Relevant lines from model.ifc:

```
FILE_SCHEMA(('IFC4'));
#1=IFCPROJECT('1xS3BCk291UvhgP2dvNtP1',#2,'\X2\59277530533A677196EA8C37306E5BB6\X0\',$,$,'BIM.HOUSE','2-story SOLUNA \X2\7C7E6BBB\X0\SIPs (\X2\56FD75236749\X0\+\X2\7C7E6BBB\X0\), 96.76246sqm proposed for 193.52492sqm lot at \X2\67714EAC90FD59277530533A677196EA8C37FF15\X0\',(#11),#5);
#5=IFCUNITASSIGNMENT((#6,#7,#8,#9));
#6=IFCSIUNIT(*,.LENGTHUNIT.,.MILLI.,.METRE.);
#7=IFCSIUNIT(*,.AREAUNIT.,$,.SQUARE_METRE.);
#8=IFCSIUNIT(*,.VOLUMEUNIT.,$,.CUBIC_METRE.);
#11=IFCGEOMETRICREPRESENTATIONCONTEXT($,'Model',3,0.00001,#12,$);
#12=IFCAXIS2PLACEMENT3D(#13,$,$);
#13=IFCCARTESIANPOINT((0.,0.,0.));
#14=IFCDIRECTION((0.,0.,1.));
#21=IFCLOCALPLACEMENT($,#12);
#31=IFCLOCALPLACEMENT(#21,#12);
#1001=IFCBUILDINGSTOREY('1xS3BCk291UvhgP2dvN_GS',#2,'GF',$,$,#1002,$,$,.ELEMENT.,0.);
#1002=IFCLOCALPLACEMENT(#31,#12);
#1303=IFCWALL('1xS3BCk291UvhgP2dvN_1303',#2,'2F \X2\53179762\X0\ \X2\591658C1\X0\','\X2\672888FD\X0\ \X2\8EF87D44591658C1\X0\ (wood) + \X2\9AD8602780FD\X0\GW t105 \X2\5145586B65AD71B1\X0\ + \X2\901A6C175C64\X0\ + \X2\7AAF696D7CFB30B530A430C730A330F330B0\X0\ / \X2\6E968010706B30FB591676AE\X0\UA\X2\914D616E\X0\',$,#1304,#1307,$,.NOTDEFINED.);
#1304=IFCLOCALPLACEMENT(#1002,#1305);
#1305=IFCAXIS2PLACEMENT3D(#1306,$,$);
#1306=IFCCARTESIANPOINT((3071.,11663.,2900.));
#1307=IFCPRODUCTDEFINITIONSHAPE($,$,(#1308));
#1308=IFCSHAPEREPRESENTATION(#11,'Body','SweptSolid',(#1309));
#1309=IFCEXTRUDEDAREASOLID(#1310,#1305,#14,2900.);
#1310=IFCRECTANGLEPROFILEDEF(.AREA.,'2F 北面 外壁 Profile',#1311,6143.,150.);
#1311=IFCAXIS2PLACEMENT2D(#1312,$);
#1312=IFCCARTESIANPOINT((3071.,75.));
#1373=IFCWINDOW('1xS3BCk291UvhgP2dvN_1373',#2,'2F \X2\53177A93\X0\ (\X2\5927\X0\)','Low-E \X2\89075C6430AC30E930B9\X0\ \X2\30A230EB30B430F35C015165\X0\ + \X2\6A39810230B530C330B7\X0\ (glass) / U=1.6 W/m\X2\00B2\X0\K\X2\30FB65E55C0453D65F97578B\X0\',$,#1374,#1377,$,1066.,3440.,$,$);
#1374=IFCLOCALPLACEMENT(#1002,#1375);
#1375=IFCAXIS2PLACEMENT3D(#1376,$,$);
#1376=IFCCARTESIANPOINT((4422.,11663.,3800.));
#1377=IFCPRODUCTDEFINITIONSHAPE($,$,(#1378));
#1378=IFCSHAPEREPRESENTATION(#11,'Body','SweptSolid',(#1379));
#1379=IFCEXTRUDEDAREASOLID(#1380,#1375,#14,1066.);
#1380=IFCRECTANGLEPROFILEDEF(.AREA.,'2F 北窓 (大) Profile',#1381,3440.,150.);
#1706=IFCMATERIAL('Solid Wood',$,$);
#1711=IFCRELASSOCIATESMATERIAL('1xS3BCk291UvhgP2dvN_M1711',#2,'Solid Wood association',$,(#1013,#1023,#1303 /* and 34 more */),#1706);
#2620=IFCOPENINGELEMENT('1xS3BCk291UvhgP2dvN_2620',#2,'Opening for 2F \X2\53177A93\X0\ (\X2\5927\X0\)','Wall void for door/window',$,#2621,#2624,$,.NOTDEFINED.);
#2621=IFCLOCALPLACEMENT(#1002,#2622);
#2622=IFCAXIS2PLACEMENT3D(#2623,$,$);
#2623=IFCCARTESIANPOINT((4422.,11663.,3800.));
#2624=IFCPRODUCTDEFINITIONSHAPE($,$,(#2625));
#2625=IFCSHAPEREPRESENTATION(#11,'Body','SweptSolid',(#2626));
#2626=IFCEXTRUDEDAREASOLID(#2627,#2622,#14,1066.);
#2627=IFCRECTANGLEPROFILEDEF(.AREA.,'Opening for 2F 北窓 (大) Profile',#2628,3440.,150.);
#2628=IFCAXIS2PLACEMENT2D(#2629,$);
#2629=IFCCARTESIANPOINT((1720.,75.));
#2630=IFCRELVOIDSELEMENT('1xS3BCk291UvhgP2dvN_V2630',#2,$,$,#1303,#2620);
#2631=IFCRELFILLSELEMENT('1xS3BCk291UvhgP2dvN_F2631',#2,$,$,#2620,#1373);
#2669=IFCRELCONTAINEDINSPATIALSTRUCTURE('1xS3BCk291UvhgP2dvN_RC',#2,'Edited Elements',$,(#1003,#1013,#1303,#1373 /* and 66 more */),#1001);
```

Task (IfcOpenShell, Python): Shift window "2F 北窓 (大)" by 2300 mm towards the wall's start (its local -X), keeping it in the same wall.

```python
import ifcopenshell
import ifcopenshell.api.geometry
import ifcopenshell.util.placement
import ifcopenshell.util.unit

model = ifcopenshell.open("model.ifc")
unit_scale = ifcopenshell.util.unit.calculate_unit_scale(model)

window = model.by_guid("1xS3BCk291UvhgP2dvN_1373")
opening = window.FillsVoids[0].RelatingOpeningElement
wall = opening.VoidsElements[0].RelatingBuildingElement

wall_matrix = ifcopenshell.util.placement.get_local_placement(wall.ObjectPlacement)
shift = wall_matrix[:3, 0] * -2.3 / unit_scale
before = ifcopenshell.util.placement.get_local_placement(window.ObjectPlacement)[:3, 3].copy()

# The window is not placed relative to its opening, so move both.
for product in (opening, window):
    matrix = ifcopenshell.util.placement.get_local_placement(product.ObjectPlacement)
    matrix[:3, 3] += shift
    ifcopenshell.api.geometry.edit_object_placement(model, product=product, matrix=matrix, is_si=False)

after = ifcopenshell.util.placement.get_local_placement(window.ObjectPlacement)[:3, 3]
print("window moved by", (after - before).round(3) + 0.0)

model.write("model_rev.ifc")
```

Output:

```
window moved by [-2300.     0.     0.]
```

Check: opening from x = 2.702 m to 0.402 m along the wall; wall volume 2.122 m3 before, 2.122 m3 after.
